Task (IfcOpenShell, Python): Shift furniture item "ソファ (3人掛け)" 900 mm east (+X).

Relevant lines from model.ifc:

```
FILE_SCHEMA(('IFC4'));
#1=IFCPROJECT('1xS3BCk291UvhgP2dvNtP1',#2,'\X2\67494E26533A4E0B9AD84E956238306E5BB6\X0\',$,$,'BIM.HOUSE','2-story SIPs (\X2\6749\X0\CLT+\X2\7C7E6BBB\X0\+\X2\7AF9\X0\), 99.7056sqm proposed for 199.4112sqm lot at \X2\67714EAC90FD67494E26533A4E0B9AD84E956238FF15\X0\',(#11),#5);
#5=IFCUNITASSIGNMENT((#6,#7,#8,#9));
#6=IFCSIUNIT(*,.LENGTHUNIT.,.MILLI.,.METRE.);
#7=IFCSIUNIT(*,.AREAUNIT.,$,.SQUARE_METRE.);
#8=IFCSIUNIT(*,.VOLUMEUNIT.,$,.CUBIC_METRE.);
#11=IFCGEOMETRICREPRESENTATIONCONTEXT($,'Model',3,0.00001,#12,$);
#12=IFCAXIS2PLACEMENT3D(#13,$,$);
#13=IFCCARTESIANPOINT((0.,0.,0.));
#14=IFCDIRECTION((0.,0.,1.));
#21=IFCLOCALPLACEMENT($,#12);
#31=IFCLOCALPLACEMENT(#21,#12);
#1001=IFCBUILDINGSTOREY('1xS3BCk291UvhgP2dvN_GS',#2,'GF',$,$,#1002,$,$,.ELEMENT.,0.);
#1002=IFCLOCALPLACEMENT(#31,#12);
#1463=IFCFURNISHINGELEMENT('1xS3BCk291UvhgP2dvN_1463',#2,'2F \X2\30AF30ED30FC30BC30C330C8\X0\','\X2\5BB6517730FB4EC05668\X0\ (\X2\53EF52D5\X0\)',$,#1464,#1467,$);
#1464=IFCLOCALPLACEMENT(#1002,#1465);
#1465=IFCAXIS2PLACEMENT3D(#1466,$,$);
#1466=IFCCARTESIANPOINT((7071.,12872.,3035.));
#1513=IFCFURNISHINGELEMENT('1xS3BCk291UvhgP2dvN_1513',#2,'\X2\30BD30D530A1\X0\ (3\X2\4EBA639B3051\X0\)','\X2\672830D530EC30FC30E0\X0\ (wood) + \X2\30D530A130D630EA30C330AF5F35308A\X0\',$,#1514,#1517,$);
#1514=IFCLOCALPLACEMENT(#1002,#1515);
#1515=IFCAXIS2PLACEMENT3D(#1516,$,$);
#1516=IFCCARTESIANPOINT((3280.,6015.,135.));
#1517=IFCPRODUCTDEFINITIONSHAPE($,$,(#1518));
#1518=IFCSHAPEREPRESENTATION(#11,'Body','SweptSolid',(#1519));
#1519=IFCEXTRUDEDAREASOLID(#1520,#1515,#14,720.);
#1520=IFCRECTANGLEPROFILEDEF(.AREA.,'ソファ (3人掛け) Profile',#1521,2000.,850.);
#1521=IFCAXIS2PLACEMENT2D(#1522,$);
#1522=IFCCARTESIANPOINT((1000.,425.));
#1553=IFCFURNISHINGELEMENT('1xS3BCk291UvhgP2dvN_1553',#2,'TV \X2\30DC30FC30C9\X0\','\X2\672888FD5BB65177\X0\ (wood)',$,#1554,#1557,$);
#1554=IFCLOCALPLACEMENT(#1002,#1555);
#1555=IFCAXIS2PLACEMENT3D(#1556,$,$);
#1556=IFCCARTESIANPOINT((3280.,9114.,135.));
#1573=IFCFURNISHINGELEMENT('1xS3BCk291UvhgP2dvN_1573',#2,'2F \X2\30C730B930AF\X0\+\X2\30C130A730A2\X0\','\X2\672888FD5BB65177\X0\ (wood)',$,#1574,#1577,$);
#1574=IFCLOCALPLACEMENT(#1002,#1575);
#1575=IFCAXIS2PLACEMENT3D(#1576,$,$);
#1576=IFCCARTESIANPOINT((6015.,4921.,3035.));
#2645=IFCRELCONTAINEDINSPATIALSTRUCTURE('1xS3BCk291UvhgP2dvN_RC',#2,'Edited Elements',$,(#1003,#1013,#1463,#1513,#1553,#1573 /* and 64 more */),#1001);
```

```python
import ifcopenshell
import ifcopenshell.api.geometry
import ifcopenshell.util.placement
import ifcopenshell.util.unit

model = ifcopenshell.open("model.ifc")
unit_scale = ifcopenshell.util.unit.calculate_unit_scale(model)

item = model.by_guid("1xS3BCk291UvhgP2dvN_1513")
matrix = ifcopenshell.util.placement.get_local_placement(item.ObjectPlacement)
matrix[0, 3] += 0.9 / unit_scale
ifcopenshell.api.geometry.edit_object_placement(model, product=item, matrix=matrix, is_si=False)

print(ifcopenshell.util.placement.get_local_placement(item.ObjectPlacement).round(3) + 0.0)

model.write("model_updated.ifc")
```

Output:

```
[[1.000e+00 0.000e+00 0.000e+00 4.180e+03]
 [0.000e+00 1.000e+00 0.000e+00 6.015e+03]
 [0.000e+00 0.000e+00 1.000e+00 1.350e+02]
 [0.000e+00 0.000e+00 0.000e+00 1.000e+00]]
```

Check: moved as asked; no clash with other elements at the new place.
